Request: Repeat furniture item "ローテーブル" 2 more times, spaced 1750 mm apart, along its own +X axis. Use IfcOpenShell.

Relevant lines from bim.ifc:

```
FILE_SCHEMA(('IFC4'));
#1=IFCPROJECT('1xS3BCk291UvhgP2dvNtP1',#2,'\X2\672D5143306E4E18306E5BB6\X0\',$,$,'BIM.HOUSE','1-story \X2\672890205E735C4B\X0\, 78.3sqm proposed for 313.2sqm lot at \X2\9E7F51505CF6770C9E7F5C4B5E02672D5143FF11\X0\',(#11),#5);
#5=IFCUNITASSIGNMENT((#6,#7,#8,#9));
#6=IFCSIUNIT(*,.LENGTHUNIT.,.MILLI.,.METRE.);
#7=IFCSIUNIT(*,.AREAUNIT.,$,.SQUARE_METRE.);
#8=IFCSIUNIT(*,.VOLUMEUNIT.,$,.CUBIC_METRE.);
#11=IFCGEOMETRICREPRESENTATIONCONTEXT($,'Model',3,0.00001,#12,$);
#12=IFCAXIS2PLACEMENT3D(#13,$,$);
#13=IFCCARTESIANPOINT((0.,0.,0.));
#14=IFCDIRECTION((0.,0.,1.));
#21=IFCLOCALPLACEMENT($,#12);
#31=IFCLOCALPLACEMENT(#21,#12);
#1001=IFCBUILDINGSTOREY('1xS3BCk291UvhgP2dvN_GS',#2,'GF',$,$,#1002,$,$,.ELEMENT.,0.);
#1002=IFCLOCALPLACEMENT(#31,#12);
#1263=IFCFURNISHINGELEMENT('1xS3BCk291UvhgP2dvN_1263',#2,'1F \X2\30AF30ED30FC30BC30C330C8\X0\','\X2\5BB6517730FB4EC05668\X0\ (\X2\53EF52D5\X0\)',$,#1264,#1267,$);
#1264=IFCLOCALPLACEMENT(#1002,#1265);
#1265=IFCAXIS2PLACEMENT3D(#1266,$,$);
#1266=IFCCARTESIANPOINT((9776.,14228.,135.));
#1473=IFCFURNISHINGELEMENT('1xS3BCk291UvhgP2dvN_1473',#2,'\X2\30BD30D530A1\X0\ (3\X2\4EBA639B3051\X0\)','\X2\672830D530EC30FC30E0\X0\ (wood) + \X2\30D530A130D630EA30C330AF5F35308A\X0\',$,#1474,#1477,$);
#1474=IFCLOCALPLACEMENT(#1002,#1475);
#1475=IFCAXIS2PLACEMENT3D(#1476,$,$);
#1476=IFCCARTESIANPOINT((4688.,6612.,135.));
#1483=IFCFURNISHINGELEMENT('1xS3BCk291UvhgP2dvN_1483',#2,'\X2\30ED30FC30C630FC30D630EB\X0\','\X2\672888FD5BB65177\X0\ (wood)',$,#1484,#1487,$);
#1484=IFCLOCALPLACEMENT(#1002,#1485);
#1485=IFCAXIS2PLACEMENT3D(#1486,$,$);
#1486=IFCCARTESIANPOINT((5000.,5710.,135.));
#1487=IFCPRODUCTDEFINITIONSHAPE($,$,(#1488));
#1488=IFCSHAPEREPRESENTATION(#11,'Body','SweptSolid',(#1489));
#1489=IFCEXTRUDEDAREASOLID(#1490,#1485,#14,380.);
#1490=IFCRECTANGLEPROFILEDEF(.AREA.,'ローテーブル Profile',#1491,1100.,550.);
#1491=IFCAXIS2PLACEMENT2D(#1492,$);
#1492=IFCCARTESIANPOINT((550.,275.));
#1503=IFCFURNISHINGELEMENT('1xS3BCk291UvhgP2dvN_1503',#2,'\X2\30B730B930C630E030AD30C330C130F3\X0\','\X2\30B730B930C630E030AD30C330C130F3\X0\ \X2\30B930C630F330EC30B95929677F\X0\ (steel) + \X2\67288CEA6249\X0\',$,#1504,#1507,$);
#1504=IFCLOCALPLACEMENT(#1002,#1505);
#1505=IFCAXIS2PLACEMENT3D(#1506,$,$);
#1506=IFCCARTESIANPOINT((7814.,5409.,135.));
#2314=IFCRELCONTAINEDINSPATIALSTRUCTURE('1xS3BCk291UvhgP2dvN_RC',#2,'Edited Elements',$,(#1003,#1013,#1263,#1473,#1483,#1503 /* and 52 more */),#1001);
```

```python
import ifcopenshell
import ifcopenshell.api.geometry
import ifcopenshell.api.root
import ifcopenshell.util.element
import ifcopenshell.util.placement
import ifcopenshell.util.unit

model = ifcopenshell.open("bim.ifc")
unit_scale = ifcopenshell.util.unit.calculate_unit_scale(model)


def reuse_history(source, copy):
    """copy_class also copies each property set's owner history, people and application; keep the originals."""
    for rel in copy.IsDefinedBy:
        if rel.is_a("IfcRelDefinesByProperties") and (history := rel.RelatingPropertyDefinition.OwnerHistory):
            rel.RelatingPropertyDefinition.OwnerHistory = source.OwnerHistory
            ifcopenshell.util.element.remove_deep2(model, history)


source = model.by_guid("1xS3BCk291UvhgP2dvN_1483")
base = ifcopenshell.util.placement.get_local_placement(source.ObjectPlacement)
step = base[:3, 0] * 1.75 / unit_scale

for i in range(1, 3):
    copy = ifcopenshell.api.root.copy_class(model, product=source)
    copy.Representation = ifcopenshell.util.element.copy_deep(
        model, source.Representation, exclude=["IfcGeometricRepresentationContext", "IfcRepresentationMap"]
    )
    reuse_history(source, copy)
    matrix = base.copy()
    matrix[:3, 3] += i * step
    print("added at", matrix[:3, 3].round(3) + 0.0)
    ifcopenshell.api.geometry.edit_object_placement(model, product=copy, matrix=matrix, is_si=False)

model.write("bim_v2.ifc")
```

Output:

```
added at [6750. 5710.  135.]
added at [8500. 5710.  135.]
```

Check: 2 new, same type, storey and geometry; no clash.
